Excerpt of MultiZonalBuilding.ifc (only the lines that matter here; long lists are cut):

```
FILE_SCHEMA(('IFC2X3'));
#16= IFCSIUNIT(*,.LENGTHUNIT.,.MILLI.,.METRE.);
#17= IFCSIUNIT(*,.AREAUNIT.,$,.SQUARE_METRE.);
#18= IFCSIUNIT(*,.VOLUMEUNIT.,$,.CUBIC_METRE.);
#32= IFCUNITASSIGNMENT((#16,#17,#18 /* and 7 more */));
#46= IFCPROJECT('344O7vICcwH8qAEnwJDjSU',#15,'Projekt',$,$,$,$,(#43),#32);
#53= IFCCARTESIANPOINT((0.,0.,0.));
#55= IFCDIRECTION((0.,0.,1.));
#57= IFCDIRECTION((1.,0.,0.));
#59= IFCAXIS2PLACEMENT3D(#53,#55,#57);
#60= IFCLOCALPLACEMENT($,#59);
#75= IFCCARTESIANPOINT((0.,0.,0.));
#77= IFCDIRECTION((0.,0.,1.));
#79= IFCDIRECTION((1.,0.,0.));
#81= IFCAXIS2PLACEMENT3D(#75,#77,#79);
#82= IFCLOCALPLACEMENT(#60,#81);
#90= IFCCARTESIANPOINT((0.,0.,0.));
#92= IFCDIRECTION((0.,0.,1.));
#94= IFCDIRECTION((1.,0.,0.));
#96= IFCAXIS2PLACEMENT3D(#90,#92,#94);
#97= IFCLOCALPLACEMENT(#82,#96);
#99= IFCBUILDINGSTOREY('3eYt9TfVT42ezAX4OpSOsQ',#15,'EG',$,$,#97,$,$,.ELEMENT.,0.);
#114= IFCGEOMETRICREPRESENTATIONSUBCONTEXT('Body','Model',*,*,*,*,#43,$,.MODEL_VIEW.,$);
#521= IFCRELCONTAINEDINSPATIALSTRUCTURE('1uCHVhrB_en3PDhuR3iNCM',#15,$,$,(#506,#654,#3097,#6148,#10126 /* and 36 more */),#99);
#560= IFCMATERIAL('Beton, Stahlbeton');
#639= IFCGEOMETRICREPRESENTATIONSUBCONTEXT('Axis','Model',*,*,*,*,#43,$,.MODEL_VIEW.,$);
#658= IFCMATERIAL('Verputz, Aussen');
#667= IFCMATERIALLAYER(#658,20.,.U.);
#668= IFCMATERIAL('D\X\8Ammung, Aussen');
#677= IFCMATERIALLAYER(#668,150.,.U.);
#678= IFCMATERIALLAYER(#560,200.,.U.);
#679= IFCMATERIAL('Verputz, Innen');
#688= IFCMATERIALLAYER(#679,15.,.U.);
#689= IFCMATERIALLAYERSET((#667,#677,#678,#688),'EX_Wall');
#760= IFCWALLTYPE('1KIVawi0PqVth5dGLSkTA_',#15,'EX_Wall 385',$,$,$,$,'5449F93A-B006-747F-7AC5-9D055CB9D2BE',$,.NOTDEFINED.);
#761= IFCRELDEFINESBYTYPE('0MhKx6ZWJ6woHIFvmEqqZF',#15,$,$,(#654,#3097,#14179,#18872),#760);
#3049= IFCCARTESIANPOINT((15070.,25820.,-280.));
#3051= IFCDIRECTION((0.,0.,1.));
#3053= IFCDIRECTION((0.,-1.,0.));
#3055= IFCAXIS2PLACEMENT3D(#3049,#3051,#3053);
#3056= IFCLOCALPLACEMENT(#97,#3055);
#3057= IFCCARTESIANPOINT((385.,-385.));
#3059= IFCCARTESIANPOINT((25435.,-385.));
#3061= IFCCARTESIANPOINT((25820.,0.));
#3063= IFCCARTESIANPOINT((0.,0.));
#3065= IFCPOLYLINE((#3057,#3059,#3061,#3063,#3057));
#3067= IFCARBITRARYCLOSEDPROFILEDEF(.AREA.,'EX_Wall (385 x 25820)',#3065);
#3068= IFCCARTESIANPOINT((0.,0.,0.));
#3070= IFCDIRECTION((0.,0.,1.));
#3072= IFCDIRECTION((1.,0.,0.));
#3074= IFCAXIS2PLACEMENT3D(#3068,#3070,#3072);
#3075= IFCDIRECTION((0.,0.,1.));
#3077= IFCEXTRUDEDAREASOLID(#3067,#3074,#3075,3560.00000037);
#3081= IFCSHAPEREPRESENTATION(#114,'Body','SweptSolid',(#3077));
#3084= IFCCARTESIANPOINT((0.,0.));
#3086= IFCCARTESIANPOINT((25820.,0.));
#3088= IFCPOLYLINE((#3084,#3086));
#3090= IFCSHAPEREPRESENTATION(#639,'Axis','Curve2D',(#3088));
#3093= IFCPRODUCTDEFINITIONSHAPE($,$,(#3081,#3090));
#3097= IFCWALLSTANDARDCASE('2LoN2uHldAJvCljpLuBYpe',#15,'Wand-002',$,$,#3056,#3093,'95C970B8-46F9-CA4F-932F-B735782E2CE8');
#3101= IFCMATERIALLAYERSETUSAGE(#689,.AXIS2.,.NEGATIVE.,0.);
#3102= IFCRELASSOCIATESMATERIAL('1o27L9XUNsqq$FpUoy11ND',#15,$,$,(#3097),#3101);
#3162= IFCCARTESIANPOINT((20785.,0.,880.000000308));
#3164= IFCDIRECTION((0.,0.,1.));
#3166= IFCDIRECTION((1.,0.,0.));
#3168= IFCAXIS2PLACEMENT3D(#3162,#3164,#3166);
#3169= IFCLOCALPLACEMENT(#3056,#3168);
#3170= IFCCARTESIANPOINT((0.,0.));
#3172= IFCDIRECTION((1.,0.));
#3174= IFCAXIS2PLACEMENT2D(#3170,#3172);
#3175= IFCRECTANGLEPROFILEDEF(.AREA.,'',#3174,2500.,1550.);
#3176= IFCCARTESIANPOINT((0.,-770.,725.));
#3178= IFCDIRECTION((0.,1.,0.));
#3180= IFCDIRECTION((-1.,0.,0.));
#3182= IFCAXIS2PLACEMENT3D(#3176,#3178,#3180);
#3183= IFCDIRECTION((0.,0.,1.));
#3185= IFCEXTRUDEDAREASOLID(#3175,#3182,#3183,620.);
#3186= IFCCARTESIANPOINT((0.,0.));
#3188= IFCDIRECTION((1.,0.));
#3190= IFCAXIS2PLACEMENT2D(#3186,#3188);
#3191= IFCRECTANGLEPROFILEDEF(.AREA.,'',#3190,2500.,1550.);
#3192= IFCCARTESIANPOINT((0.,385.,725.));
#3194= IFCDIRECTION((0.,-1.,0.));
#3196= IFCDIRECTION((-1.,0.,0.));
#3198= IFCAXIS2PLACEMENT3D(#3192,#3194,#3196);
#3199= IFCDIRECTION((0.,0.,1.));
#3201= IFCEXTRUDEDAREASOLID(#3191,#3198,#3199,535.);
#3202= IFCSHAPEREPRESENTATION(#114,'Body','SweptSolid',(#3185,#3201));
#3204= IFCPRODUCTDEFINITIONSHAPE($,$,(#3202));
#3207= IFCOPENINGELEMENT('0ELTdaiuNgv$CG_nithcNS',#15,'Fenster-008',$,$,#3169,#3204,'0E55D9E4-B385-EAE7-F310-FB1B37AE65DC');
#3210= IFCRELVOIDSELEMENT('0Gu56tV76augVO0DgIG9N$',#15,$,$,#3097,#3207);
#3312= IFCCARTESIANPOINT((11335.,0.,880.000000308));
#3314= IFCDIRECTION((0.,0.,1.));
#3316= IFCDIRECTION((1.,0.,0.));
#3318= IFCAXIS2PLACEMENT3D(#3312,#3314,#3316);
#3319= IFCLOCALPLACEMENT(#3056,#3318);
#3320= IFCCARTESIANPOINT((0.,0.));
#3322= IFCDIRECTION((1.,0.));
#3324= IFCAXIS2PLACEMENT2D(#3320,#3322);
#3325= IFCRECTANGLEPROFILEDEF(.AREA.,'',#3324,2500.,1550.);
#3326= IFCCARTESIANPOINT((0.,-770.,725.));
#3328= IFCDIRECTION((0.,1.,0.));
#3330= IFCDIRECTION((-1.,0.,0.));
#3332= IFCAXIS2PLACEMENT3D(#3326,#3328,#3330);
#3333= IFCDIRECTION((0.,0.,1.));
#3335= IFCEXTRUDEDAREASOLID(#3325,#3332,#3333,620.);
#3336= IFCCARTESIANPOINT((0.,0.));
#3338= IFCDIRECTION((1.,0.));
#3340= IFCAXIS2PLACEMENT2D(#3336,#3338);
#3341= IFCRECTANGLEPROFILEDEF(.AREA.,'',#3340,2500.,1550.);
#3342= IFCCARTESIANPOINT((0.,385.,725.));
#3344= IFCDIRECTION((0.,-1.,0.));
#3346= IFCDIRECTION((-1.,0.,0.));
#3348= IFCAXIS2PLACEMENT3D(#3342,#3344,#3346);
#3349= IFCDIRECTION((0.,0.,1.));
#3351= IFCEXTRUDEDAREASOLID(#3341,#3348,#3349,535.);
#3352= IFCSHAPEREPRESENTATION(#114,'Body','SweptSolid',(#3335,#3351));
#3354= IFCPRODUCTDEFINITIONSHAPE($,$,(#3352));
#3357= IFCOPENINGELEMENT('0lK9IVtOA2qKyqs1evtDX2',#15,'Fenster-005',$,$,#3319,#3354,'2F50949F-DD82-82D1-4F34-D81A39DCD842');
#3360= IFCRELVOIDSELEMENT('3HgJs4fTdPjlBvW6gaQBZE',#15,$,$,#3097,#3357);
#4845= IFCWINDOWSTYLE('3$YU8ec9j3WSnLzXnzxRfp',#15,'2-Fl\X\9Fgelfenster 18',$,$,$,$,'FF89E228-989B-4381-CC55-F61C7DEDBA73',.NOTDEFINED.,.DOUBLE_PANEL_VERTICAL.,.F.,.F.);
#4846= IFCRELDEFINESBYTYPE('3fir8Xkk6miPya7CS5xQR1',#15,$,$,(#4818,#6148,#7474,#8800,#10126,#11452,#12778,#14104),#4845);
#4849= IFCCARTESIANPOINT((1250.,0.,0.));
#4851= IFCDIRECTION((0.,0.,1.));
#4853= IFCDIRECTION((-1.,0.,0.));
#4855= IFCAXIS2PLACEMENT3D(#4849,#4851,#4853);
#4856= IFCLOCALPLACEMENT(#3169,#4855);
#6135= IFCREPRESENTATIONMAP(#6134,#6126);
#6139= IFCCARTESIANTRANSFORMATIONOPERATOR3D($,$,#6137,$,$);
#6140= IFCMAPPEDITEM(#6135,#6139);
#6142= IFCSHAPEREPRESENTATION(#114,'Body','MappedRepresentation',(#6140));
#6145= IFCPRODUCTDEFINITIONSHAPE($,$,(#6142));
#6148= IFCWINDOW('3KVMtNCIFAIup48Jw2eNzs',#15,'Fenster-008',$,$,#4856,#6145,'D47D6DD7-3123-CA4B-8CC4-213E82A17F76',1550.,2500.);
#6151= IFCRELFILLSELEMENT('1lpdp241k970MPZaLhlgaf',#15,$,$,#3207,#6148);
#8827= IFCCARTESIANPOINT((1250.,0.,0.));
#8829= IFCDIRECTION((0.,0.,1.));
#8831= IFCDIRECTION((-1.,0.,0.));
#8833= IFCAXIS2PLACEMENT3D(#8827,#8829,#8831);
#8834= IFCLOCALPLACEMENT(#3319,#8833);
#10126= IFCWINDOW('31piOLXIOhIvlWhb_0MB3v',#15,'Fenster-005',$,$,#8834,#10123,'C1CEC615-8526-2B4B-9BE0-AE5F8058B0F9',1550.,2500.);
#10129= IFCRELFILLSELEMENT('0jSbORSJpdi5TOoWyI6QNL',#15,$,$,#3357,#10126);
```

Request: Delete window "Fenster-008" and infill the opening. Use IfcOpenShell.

```python
import ifcopenshell
import ifcopenshell.api.feature
import ifcopenshell.api.root
import ifcopenshell.geom
import ifcopenshell.util.shape

model = ifcopenshell.open("MultiZonalBuilding.ifc")
settings = ifcopenshell.geom.settings()


def volume(element):
    """Net volume in cubic metres, openings subtracted."""
    shape = ifcopenshell.geom.create_shape(settings, element)
    return ifcopenshell.util.shape.get_volume(shape.geometry)


window = model.by_guid("3KVMtNCIFAIup48Jw2eNzs")
opening = window.FillsVoids[0].RelatingOpeningElement
wall = opening.VoidsElements[0].RelatingBuildingElement
before = volume(wall)

ifcopenshell.api.root.remove_product(model, product=window)
ifcopenshell.api.feature.remove_feature(model, feature=opening)

after = volume(wall)

print(f"wall volume {before:.3f} -> {after:.3f} m3")

model.write("MultiZonalBuilding_updated.ifc")
```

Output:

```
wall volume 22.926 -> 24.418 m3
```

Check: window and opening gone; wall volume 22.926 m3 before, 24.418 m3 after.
